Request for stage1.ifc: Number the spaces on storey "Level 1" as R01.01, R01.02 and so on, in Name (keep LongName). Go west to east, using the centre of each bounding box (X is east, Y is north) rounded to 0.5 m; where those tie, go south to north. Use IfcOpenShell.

First a look at what the model holds.

```python
import ifcopenshell
import ifcopenshell.util.element
import ifcopenshell.util.placement

model = ifcopenshell.open("stage1.ifc")
print(model.schema)
storey = next(s for s in model.by_type("IfcBuildingStorey") if s.Name == "Level 1")
spaces = [e for e in ifcopenshell.util.element.get_decomposition(storey) if e.is_a("IfcSpace")]
for e in sorted(spaces, key=lambda e: e.id()):
    origin = ifcopenshell.util.placement.get_local_placement(e.ObjectPlacement)[:3, 3]
    print(e.id(), e.Name, e.LongName, origin.round(2) + 0.0, sep=" | ")
```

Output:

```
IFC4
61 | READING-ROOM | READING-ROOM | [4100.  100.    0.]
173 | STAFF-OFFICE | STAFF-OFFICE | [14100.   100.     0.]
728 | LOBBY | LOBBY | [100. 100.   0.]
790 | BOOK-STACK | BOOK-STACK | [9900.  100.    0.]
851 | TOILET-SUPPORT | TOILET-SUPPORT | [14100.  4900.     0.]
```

```python
import ifcopenshell
import ifcopenshell.geom
import ifcopenshell.util.element
import ifcopenshell.util.shape

model = ifcopenshell.open("stage1.ifc")
settings = ifcopenshell.geom.settings()
settings.set("use-world-coords", True)


def centre(element):
    shape = ifcopenshell.geom.create_shape(settings, element)
    return ifcopenshell.util.shape.get_bbox_centroid(shape.geometry)


storey = next(s for s in model.by_type("IfcBuildingStorey") if s.Name == "Level 1")
spaces = [e for e in ifcopenshell.util.element.get_decomposition(storey) if e.is_a("IfcSpace")]

# Insertion points can sit at a corner or the storey origin, so sort by the geometry (in metres).
centres = {e: centre(e) for e in spaces}
spaces.sort(key=lambda e: (round(centres[e][0] / 0.5), centres[e][1]))

for i, e in enumerate(spaces, start=1):
    number = f"R01.{i:02d}"
    e.Name = number
    print(e.id(), number)

model.write("stage1_rev.ifc")
```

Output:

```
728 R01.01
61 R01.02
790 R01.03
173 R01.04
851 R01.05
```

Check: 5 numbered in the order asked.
